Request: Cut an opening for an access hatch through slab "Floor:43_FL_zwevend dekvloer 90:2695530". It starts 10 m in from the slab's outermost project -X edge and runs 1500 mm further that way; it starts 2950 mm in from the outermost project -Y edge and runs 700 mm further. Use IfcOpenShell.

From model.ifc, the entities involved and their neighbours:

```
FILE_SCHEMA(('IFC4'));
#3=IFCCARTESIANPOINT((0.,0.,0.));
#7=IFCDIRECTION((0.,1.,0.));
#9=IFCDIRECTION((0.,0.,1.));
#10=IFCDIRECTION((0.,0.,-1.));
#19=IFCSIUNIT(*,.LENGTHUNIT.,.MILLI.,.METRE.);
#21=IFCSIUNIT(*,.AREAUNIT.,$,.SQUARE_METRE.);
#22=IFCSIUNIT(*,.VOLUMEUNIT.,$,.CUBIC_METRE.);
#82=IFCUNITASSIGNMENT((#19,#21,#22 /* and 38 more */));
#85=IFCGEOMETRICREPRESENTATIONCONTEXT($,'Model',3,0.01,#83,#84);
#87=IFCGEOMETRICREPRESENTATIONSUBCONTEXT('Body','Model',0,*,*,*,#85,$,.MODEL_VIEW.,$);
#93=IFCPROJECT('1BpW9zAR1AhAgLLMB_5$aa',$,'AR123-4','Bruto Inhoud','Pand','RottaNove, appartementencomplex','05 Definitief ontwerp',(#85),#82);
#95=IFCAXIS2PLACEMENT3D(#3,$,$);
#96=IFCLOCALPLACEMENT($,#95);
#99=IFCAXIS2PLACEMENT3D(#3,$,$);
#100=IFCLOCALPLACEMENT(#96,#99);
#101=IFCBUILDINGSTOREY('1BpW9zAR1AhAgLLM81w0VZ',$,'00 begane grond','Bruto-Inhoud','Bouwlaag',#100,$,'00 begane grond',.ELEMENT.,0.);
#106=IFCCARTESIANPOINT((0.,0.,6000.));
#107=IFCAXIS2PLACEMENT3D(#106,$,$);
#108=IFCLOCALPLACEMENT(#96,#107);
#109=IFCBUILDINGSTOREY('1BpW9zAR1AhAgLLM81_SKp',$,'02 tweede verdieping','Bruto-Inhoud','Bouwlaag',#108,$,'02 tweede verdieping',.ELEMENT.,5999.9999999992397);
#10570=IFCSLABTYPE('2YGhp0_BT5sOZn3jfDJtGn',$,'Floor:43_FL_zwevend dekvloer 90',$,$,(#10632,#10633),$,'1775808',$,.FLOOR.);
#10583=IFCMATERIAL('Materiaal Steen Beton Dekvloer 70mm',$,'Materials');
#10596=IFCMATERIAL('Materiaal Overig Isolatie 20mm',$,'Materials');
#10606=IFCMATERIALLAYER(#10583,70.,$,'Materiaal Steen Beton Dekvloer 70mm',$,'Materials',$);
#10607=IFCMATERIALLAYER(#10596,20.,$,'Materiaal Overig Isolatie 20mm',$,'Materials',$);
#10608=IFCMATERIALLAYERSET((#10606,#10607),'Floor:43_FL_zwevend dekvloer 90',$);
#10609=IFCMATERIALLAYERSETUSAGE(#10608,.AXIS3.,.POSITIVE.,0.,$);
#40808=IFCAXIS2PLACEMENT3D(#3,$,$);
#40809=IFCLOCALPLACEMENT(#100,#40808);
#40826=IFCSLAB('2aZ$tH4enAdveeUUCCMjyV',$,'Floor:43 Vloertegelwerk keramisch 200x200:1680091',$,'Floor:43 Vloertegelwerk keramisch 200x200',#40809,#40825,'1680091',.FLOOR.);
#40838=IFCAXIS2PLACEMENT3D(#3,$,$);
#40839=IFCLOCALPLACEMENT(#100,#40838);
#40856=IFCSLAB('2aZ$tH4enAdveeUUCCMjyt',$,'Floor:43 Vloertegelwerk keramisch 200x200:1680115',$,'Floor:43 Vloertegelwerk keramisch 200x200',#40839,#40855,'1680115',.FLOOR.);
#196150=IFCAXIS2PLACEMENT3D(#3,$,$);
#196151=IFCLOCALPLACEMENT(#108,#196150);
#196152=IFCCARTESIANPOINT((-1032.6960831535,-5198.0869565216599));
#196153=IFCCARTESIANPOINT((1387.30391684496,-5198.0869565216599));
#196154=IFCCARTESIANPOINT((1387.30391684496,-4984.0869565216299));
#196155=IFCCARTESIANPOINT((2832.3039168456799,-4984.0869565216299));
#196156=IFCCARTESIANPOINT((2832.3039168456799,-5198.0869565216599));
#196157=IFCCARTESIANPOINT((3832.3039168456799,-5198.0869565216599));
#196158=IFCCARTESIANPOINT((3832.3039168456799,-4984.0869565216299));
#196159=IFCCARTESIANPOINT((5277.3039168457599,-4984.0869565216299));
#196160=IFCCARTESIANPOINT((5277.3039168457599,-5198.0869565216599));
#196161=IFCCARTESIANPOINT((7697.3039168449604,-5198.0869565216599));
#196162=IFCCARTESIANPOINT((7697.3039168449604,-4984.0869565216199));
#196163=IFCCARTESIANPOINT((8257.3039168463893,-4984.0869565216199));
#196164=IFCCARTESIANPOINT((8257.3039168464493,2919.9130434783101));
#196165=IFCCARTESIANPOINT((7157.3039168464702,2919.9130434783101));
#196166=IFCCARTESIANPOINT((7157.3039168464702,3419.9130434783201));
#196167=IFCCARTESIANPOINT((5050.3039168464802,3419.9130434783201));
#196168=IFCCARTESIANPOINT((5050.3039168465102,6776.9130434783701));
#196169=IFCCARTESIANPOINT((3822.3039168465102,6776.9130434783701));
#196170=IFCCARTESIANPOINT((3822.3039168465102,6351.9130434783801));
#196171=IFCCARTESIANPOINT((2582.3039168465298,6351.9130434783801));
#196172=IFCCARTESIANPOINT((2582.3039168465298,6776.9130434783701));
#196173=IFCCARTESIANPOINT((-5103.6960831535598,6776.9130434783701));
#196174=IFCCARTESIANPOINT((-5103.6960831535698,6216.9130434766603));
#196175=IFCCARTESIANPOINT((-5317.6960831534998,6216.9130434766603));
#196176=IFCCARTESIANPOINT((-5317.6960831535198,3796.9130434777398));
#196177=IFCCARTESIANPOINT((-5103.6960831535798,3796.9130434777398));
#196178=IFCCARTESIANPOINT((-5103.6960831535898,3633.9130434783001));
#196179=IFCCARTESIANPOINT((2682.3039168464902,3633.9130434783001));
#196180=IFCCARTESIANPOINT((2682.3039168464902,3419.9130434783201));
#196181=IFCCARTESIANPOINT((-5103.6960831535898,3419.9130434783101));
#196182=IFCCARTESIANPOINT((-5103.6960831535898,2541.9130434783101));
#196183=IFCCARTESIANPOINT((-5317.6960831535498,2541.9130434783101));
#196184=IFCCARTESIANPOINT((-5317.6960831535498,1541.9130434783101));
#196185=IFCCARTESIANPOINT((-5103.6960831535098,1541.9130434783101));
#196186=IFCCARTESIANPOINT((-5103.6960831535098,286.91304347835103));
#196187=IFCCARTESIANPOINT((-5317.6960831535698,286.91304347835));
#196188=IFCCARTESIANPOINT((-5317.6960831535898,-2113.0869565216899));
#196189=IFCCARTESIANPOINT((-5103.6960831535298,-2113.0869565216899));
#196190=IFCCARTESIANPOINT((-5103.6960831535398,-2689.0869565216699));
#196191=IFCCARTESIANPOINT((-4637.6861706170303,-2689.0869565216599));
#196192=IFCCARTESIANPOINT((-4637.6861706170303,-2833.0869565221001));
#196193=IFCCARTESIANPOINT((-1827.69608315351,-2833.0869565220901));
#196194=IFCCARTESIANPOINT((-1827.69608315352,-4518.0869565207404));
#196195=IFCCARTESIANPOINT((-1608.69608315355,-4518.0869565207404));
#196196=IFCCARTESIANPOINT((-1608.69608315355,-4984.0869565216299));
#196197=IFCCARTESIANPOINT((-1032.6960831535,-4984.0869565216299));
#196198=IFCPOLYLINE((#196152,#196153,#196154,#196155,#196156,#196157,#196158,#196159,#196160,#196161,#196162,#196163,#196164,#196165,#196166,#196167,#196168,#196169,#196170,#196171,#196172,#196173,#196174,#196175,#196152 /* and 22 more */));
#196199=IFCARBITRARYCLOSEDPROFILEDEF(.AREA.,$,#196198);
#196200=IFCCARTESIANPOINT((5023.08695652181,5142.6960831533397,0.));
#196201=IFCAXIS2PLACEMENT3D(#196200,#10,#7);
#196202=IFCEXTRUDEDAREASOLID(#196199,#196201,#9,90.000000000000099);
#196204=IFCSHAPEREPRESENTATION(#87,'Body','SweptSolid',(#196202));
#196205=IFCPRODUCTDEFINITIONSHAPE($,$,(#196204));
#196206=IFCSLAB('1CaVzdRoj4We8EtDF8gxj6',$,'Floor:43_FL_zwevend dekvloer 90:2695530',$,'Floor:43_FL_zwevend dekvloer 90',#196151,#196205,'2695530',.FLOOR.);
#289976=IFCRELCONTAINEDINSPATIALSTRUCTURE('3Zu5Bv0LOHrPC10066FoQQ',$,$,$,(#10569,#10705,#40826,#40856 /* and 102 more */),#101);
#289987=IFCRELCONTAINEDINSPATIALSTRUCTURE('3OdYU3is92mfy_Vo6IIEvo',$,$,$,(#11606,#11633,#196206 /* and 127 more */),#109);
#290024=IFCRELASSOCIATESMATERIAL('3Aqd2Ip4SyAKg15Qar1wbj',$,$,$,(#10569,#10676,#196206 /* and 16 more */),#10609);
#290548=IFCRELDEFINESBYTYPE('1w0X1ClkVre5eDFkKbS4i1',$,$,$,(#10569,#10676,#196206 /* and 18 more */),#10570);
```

```python
import numpy as np
import ifcopenshell
import ifcopenshell.api.feature
import ifcopenshell.api.geometry
import ifcopenshell.api.root
import ifcopenshell.geom
import ifcopenshell.util.placement
import ifcopenshell.util.representation
import ifcopenshell.util.shape
import ifcopenshell.util.unit

model = ifcopenshell.open("model.ifc")
unit_scale = ifcopenshell.util.unit.calculate_unit_scale(model)
settings = ifcopenshell.geom.settings()


def volume(element):
    """Net volume in cubic metres, openings subtracted."""
    shape = ifcopenshell.geom.create_shape(settings, element)
    return ifcopenshell.util.shape.get_volume(shape.geometry)


slab = model.by_guid("1CaVzdRoj4We8EtDF8gxj6")
before = volume(slab)

# Extent in the slab's own axes, in metres. The edges named are its -X and -Y sides.
slab_shape = ifcopenshell.geom.create_shape(settings, slab)
vertices = ifcopenshell.util.shape.get_vertices(slab_shape.geometry)
x_min, y_min, bottom = vertices.min(axis=0)
top = vertices[:, 2].max()

opening = ifcopenshell.api.root.create_entity(model, ifc_class="IfcOpeningElement", name="Access hatch opening", predefined_type="OPENING")
context = ifcopenshell.util.representation.get_context(model, "Model", "Body", "MODEL_VIEW")
width, depth = 1.5, 0.7
outline = [(0.0, 0.0), (width, 0.0), (width, depth), (0.0, depth), (0.0, 0.0)]
# Overshoot both faces by 50 mm so the cut is clean.
shape = ifcopenshell.api.geometry.add_slab_representation(
    model, context=context, depth=top - bottom + 0.1, polyline=outline
)
ifcopenshell.api.geometry.assign_representation(model, product=opening, representation=shape)

matrix = ifcopenshell.util.placement.get_local_placement(slab.ObjectPlacement)
matrix[:, 3] = matrix @ np.append(np.array([x_min + 10, y_min + 2.95, bottom - 0.05]) / unit_scale, 1.0)
ifcopenshell.api.geometry.edit_object_placement(model, product=opening, matrix=matrix, is_si=False)
ifcopenshell.api.feature.add_feature(model, feature=opening, element=slab)

after = volume(slab)

print(f"slab volume {before:.3f} -> {after:.3f} m3")

model.write("model_rev.ifc")
```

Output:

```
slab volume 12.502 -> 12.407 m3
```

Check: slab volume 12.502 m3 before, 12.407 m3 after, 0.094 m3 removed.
